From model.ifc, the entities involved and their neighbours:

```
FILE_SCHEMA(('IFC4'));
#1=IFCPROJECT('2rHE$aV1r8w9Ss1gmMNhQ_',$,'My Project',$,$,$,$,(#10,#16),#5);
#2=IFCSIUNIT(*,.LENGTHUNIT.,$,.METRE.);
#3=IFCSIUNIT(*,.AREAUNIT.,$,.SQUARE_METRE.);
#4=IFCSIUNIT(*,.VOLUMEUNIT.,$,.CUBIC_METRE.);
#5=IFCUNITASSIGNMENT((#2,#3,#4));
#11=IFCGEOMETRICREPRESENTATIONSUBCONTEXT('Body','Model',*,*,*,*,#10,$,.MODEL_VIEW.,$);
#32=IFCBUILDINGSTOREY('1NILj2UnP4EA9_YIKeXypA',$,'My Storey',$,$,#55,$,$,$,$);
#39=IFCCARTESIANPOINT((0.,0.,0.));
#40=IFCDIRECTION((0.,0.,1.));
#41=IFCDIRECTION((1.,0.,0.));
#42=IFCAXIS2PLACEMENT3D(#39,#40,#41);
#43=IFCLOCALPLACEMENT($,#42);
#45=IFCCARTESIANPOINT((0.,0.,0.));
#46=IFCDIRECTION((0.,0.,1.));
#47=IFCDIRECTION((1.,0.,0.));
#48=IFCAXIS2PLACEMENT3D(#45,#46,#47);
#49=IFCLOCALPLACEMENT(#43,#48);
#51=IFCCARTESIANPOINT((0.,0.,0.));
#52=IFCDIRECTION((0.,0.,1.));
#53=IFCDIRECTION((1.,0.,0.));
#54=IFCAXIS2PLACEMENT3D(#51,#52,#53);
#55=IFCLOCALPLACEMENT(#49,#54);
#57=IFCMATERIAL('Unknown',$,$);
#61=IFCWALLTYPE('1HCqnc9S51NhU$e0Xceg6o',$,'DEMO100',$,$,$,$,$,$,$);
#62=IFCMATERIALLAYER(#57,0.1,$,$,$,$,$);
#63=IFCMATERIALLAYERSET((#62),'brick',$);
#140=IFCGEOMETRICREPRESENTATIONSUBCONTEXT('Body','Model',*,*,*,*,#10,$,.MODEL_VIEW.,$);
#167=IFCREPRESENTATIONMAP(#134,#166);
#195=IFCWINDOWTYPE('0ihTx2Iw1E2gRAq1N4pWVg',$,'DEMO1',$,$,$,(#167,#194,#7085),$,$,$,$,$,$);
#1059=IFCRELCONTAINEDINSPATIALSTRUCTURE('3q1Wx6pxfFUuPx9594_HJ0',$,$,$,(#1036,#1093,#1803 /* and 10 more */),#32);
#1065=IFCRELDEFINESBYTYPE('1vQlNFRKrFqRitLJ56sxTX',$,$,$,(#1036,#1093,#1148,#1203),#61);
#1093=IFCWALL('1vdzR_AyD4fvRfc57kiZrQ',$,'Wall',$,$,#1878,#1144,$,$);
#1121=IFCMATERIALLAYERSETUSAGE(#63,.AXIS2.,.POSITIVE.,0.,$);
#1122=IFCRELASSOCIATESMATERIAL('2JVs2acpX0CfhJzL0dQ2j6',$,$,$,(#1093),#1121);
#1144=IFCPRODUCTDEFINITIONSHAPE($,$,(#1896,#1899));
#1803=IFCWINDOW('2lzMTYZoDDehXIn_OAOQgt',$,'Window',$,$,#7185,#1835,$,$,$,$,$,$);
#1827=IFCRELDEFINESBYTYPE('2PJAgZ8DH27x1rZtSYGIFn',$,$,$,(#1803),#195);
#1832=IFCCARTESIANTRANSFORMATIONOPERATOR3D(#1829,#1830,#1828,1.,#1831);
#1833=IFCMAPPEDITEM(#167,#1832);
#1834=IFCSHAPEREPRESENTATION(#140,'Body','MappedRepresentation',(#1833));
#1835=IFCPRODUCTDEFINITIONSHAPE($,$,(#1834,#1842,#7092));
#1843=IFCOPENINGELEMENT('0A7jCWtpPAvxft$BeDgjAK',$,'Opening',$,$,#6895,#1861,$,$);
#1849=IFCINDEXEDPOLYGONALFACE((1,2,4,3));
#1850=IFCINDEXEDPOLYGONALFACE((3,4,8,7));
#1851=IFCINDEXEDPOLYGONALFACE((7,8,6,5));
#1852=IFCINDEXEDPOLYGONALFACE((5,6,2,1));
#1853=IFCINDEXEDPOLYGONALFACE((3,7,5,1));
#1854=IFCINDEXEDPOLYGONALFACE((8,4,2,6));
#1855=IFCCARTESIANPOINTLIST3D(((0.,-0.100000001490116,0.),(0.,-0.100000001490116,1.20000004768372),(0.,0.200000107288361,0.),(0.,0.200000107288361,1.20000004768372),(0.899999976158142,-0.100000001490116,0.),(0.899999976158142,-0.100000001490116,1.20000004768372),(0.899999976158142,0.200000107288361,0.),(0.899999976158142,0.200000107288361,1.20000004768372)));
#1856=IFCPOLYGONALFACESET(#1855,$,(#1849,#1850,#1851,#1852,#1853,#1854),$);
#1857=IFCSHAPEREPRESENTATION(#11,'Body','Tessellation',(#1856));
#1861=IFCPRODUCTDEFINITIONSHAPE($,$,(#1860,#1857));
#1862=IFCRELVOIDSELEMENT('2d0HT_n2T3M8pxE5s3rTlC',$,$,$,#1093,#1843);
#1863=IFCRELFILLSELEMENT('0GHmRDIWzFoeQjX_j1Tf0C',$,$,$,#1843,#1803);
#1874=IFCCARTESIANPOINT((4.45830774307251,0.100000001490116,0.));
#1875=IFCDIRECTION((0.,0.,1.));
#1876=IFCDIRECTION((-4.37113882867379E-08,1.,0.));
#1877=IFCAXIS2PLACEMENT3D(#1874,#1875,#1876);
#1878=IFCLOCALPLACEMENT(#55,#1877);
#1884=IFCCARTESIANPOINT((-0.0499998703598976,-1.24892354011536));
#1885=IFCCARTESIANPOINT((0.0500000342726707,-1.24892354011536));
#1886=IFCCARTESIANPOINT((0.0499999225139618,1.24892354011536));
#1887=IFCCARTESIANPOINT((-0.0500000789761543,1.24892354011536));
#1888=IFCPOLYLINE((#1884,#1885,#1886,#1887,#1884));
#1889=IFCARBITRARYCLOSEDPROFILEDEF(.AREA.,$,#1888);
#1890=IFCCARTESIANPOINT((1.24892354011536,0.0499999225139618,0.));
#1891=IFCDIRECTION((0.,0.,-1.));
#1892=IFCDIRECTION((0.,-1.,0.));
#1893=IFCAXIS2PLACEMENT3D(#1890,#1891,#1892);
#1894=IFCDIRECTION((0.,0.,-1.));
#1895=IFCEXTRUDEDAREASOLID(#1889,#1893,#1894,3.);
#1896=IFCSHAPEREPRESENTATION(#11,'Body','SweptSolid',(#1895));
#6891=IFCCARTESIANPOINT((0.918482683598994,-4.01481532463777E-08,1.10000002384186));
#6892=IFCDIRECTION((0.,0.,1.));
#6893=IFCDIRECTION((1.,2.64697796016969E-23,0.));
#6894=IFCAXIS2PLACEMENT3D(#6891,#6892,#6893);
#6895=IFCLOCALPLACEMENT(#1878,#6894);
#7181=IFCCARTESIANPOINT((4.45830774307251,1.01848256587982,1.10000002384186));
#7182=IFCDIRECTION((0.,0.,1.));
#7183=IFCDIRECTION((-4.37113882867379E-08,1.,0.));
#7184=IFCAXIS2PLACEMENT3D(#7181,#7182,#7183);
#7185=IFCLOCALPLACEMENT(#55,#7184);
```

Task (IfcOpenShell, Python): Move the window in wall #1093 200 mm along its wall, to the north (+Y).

```python
import ifcopenshell
import ifcopenshell.api.geometry
import ifcopenshell.util.placement

model = ifcopenshell.open("model.ifc")

window = model.by_id(1803)
opening = window.FillsVoids[0].RelatingOpeningElement
wall = opening.VoidsElements[0].RelatingBuildingElement

wall_matrix = ifcopenshell.util.placement.get_local_placement(wall.ObjectPlacement)
shift = wall_matrix[:3, 0] * 0.2
before = ifcopenshell.util.placement.get_local_placement(window.ObjectPlacement)[:3, 3].copy()

# The window is not placed relative to its opening, so move both.
for product in (opening, window):
    matrix = ifcopenshell.util.placement.get_local_placement(product.ObjectPlacement)
    matrix[:3, 3] += shift
    ifcopenshell.api.geometry.edit_object_placement(model, product=product, matrix=matrix, is_si=False)

after = ifcopenshell.util.placement.get_local_placement(window.ObjectPlacement)[:3, 3]
print("window moved by", (after - before).round(3) + 0.0)

model.write("model_v2.ifc")
```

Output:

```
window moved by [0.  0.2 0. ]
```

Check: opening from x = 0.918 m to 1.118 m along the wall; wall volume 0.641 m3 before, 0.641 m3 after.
